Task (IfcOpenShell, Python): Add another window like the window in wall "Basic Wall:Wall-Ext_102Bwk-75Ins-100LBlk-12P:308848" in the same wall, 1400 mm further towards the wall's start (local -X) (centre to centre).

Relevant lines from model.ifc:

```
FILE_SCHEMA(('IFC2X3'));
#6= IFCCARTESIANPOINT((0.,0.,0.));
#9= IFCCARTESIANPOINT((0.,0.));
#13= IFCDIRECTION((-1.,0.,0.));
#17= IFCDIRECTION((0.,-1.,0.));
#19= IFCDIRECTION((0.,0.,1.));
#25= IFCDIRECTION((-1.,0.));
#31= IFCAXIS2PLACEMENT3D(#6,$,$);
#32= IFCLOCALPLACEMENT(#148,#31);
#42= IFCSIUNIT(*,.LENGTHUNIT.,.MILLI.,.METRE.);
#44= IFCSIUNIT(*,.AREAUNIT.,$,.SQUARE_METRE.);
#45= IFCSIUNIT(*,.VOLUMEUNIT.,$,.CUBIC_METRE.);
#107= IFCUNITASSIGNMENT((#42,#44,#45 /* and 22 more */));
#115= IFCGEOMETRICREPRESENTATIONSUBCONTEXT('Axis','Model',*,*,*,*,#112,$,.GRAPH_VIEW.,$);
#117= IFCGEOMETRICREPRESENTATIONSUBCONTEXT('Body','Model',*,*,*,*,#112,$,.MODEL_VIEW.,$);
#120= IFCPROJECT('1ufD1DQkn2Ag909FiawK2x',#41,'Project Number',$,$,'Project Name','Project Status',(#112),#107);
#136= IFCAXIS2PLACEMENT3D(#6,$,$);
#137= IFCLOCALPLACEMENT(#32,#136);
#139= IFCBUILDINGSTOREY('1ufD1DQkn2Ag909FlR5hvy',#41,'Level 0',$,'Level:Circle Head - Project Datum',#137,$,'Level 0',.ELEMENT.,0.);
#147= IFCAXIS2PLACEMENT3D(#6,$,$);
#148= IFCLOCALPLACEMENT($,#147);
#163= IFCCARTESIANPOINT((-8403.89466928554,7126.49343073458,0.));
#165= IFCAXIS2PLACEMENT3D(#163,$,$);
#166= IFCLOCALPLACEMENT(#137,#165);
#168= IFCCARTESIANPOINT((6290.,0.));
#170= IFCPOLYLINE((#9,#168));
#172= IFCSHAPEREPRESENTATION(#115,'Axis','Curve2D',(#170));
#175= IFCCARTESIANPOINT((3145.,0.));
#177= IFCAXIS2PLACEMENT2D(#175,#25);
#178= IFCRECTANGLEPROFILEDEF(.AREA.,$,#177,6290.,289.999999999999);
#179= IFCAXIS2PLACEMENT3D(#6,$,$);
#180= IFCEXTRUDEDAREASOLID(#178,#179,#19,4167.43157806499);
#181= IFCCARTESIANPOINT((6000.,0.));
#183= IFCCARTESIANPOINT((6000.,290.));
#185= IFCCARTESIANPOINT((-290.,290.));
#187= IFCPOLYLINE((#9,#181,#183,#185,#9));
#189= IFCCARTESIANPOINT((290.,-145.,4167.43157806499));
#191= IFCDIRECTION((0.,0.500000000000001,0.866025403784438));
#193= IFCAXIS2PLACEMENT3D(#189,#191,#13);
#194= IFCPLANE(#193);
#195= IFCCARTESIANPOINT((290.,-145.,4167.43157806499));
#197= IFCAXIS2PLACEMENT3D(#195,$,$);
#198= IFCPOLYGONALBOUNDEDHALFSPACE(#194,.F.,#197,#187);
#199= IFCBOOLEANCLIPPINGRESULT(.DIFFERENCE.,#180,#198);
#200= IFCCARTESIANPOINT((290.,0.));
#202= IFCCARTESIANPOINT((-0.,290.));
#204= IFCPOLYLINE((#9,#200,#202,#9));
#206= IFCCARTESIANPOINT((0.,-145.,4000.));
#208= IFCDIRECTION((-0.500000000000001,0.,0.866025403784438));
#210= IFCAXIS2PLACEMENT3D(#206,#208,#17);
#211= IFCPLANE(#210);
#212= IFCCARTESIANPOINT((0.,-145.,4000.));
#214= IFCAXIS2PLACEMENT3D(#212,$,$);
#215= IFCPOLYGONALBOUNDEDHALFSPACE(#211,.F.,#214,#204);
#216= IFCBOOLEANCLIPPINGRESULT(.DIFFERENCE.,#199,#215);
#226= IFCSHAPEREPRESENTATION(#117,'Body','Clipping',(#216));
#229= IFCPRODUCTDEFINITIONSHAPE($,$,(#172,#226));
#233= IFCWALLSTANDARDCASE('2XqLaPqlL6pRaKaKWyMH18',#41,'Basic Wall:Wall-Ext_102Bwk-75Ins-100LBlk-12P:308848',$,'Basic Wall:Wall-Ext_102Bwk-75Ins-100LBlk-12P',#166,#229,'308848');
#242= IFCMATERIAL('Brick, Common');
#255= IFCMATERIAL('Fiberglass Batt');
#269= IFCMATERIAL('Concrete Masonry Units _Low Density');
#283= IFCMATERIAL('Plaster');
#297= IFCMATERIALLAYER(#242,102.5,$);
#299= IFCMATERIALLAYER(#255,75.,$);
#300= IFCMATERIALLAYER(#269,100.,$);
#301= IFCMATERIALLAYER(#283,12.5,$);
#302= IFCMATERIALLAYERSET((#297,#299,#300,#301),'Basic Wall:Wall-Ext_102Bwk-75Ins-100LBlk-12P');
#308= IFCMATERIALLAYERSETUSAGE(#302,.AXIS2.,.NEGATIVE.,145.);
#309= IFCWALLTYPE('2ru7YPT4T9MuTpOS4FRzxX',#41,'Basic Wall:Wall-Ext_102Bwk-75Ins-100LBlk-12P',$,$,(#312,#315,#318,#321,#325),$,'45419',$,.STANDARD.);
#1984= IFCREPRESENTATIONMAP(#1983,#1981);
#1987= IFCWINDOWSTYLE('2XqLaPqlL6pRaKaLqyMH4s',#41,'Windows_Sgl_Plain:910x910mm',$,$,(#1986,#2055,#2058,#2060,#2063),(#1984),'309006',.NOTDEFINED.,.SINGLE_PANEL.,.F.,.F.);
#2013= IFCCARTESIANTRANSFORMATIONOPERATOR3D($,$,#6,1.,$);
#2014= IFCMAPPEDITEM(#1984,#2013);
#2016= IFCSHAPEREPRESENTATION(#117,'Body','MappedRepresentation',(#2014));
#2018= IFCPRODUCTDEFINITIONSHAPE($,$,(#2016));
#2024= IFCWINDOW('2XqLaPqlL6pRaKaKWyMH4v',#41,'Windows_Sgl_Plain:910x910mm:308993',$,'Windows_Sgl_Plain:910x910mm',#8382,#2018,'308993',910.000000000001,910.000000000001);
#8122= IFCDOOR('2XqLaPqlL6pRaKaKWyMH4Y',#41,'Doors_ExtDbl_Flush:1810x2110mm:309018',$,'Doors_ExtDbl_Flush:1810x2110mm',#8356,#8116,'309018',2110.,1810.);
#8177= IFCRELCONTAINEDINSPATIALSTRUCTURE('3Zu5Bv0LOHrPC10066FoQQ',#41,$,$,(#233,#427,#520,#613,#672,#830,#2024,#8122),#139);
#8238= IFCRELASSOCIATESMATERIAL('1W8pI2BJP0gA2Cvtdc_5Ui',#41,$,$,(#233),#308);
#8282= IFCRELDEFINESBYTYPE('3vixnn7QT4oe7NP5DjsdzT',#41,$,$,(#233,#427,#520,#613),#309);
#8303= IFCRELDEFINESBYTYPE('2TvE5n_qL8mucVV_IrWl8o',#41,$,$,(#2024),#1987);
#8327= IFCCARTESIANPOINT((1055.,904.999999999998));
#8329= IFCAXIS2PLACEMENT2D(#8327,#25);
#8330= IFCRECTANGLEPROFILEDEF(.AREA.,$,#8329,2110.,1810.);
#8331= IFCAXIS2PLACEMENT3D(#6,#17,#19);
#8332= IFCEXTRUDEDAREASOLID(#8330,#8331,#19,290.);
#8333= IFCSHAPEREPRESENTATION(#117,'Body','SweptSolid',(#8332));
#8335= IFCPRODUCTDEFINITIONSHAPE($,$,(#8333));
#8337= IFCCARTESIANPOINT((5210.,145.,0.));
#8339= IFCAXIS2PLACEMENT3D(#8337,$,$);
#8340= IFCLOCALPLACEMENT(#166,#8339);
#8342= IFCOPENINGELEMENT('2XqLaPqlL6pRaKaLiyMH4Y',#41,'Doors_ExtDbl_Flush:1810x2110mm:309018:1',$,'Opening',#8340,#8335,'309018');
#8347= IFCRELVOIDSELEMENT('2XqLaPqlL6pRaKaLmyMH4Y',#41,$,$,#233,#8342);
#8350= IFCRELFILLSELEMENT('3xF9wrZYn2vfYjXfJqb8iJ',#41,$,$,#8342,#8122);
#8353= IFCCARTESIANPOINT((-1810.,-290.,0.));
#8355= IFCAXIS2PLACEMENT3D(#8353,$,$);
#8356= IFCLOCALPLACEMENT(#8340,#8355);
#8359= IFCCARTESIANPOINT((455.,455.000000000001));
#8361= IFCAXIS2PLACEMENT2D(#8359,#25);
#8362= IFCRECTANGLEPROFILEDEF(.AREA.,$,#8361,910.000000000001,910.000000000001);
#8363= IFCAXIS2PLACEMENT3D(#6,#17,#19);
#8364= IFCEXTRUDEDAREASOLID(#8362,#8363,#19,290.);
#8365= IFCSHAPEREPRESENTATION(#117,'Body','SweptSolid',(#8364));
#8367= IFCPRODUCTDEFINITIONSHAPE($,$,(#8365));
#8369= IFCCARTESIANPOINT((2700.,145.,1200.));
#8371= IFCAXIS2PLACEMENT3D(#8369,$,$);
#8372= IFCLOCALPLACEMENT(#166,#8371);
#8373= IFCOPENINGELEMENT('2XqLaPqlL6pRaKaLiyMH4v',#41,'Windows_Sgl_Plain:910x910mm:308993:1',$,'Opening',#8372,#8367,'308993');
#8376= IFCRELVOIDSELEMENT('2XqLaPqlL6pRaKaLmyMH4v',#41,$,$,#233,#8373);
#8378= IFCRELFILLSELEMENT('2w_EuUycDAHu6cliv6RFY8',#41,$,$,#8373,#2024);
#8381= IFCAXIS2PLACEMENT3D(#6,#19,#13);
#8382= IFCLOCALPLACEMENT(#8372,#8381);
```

```python
import ifcopenshell
import ifcopenshell.api.feature
import ifcopenshell.api.geometry
import ifcopenshell.api.root
import ifcopenshell.geom
import ifcopenshell.util.element
import ifcopenshell.util.placement
import ifcopenshell.util.shape
import ifcopenshell.util.unit

model = ifcopenshell.open("model.ifc")
unit_scale = ifcopenshell.util.unit.calculate_unit_scale(model)
settings = ifcopenshell.geom.settings()


def volume(element):
    """Net volume in cubic metres, openings subtracted."""
    shape = ifcopenshell.geom.create_shape(settings, element)
    return ifcopenshell.util.shape.get_volume(shape.geometry)


def reuse_history(source, copy):
    """copy_class also copies each property set's owner history, people and application; keep the originals."""
    for rel in copy.IsDefinedBy:
        if rel.is_a("IfcRelDefinesByProperties") and (history := rel.RelatingPropertyDefinition.OwnerHistory):
            rel.RelatingPropertyDefinition.OwnerHistory = source.OwnerHistory
            ifcopenshell.util.element.remove_deep2(model, history)


window = model.by_guid("2XqLaPqlL6pRaKaKWyMH4v")
opening = window.FillsVoids[0].RelatingOpeningElement
wall = opening.VoidsElements[0].RelatingBuildingElement
before = volume(wall)
shift = ifcopenshell.util.placement.get_local_placement(wall.ObjectPlacement)[:3, 0] * -1.4 / unit_scale

# copy_class copies the void relationship, type, container and properties, but no geometry.
new_opening = ifcopenshell.api.root.copy_class(model, product=opening)
new_opening.Representation = ifcopenshell.util.element.copy_deep(
    model, opening.Representation, exclude=["IfcGeometricRepresentationContext", "IfcRepresentationMap"]
)
new_opening.Name = "Windows_Sgl_Plain:910x910mm"
new_opening.Tag = None
new_window = ifcopenshell.api.root.copy_class(model, product=window)
new_window.Representation = ifcopenshell.util.element.copy_deep(
    model, window.Representation, exclude=["IfcGeometricRepresentationContext", "IfcRepresentationMap"]
)
new_window.Name = "Windows_Sgl_Plain:910x910mm"
new_window.Tag = None
reuse_history(window, new_window)
fills = ifcopenshell.api.feature.add_filling(model, opening=new_opening, element=new_window)
fills.OwnerHistory = new_window.OwnerHistory  # required in IFC2X3

for old, new in ((opening, new_opening), (window, new_window)):
    matrix = ifcopenshell.util.placement.get_local_placement(old.ObjectPlacement)
    matrix[:3, 3] += shift
    ifcopenshell.api.geometry.edit_object_placement(model, product=new, matrix=matrix, is_si=False)

after = volume(wall)

print(f"wall volume {before:.3f} -> {after:.3f} m3")

model.write("model_edited.ifc")
```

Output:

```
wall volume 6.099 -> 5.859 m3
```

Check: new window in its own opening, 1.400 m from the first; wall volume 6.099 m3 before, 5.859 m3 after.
